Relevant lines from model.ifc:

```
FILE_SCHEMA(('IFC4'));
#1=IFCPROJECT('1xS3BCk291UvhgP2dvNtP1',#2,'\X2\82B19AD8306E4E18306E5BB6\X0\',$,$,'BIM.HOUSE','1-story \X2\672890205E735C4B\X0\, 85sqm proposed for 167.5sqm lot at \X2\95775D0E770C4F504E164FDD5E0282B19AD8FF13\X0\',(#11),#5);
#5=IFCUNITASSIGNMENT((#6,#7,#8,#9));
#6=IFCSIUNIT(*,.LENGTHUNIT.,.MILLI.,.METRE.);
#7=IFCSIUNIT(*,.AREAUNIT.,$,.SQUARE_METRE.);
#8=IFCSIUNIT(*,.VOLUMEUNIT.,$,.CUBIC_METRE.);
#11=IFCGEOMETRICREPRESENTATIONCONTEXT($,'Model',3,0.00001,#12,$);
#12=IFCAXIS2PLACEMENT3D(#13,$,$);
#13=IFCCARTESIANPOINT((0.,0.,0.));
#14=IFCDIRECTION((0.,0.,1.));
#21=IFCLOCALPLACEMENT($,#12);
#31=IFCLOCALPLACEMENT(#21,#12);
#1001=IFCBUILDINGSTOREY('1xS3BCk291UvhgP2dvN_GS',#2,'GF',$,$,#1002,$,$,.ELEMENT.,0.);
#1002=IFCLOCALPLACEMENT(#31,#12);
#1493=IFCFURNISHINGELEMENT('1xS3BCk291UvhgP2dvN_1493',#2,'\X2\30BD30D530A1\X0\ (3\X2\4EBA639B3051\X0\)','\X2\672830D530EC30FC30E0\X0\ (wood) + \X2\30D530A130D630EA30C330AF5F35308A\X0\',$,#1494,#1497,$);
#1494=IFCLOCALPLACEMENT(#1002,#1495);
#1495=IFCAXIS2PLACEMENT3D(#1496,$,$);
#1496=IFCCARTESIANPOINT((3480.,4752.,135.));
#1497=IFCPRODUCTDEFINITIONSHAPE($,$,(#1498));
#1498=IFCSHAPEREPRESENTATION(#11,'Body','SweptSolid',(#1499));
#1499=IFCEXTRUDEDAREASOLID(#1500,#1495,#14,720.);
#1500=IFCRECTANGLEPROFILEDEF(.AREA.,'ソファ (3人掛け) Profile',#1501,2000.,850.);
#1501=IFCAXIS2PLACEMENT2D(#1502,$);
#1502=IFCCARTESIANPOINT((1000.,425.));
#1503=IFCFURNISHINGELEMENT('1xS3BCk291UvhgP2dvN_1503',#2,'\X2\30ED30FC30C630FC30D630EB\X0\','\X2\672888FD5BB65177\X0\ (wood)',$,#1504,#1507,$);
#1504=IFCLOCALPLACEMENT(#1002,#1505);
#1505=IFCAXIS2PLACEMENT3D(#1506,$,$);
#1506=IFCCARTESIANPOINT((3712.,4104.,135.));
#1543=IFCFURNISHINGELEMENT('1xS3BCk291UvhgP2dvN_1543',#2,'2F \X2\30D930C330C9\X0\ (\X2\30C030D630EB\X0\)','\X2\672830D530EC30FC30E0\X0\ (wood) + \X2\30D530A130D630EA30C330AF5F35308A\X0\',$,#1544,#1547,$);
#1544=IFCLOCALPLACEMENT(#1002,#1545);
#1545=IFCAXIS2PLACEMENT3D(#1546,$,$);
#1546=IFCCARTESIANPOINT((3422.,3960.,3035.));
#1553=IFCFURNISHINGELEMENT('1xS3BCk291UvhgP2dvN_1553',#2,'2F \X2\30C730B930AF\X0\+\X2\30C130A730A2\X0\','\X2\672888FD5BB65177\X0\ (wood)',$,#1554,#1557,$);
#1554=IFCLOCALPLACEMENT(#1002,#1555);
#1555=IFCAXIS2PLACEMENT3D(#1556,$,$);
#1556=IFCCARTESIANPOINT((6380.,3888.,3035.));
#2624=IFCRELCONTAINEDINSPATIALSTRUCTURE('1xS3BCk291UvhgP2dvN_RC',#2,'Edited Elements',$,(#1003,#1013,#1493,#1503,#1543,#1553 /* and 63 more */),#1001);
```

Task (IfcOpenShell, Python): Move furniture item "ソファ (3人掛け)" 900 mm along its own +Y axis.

```python
import ifcopenshell
import ifcopenshell.api.geometry
import ifcopenshell.util.placement
import ifcopenshell.util.unit

model = ifcopenshell.open("model.ifc")
unit_scale = ifcopenshell.util.unit.calculate_unit_scale(model)

item = model.by_guid("1xS3BCk291UvhgP2dvN_1493")
matrix = ifcopenshell.util.placement.get_local_placement(item.ObjectPlacement)
matrix[:3, 3] += matrix[:3, 1] * 0.9 / unit_scale
ifcopenshell.api.geometry.edit_object_placement(model, product=item, matrix=matrix, is_si=False)

print(ifcopenshell.util.placement.get_local_placement(item.ObjectPlacement).round(3) + 0.0)

model.write("model_edited.ifc")
```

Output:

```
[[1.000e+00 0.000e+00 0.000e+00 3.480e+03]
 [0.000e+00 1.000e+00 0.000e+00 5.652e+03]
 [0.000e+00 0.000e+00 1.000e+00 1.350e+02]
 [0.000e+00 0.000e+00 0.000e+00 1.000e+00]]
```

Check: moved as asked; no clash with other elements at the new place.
